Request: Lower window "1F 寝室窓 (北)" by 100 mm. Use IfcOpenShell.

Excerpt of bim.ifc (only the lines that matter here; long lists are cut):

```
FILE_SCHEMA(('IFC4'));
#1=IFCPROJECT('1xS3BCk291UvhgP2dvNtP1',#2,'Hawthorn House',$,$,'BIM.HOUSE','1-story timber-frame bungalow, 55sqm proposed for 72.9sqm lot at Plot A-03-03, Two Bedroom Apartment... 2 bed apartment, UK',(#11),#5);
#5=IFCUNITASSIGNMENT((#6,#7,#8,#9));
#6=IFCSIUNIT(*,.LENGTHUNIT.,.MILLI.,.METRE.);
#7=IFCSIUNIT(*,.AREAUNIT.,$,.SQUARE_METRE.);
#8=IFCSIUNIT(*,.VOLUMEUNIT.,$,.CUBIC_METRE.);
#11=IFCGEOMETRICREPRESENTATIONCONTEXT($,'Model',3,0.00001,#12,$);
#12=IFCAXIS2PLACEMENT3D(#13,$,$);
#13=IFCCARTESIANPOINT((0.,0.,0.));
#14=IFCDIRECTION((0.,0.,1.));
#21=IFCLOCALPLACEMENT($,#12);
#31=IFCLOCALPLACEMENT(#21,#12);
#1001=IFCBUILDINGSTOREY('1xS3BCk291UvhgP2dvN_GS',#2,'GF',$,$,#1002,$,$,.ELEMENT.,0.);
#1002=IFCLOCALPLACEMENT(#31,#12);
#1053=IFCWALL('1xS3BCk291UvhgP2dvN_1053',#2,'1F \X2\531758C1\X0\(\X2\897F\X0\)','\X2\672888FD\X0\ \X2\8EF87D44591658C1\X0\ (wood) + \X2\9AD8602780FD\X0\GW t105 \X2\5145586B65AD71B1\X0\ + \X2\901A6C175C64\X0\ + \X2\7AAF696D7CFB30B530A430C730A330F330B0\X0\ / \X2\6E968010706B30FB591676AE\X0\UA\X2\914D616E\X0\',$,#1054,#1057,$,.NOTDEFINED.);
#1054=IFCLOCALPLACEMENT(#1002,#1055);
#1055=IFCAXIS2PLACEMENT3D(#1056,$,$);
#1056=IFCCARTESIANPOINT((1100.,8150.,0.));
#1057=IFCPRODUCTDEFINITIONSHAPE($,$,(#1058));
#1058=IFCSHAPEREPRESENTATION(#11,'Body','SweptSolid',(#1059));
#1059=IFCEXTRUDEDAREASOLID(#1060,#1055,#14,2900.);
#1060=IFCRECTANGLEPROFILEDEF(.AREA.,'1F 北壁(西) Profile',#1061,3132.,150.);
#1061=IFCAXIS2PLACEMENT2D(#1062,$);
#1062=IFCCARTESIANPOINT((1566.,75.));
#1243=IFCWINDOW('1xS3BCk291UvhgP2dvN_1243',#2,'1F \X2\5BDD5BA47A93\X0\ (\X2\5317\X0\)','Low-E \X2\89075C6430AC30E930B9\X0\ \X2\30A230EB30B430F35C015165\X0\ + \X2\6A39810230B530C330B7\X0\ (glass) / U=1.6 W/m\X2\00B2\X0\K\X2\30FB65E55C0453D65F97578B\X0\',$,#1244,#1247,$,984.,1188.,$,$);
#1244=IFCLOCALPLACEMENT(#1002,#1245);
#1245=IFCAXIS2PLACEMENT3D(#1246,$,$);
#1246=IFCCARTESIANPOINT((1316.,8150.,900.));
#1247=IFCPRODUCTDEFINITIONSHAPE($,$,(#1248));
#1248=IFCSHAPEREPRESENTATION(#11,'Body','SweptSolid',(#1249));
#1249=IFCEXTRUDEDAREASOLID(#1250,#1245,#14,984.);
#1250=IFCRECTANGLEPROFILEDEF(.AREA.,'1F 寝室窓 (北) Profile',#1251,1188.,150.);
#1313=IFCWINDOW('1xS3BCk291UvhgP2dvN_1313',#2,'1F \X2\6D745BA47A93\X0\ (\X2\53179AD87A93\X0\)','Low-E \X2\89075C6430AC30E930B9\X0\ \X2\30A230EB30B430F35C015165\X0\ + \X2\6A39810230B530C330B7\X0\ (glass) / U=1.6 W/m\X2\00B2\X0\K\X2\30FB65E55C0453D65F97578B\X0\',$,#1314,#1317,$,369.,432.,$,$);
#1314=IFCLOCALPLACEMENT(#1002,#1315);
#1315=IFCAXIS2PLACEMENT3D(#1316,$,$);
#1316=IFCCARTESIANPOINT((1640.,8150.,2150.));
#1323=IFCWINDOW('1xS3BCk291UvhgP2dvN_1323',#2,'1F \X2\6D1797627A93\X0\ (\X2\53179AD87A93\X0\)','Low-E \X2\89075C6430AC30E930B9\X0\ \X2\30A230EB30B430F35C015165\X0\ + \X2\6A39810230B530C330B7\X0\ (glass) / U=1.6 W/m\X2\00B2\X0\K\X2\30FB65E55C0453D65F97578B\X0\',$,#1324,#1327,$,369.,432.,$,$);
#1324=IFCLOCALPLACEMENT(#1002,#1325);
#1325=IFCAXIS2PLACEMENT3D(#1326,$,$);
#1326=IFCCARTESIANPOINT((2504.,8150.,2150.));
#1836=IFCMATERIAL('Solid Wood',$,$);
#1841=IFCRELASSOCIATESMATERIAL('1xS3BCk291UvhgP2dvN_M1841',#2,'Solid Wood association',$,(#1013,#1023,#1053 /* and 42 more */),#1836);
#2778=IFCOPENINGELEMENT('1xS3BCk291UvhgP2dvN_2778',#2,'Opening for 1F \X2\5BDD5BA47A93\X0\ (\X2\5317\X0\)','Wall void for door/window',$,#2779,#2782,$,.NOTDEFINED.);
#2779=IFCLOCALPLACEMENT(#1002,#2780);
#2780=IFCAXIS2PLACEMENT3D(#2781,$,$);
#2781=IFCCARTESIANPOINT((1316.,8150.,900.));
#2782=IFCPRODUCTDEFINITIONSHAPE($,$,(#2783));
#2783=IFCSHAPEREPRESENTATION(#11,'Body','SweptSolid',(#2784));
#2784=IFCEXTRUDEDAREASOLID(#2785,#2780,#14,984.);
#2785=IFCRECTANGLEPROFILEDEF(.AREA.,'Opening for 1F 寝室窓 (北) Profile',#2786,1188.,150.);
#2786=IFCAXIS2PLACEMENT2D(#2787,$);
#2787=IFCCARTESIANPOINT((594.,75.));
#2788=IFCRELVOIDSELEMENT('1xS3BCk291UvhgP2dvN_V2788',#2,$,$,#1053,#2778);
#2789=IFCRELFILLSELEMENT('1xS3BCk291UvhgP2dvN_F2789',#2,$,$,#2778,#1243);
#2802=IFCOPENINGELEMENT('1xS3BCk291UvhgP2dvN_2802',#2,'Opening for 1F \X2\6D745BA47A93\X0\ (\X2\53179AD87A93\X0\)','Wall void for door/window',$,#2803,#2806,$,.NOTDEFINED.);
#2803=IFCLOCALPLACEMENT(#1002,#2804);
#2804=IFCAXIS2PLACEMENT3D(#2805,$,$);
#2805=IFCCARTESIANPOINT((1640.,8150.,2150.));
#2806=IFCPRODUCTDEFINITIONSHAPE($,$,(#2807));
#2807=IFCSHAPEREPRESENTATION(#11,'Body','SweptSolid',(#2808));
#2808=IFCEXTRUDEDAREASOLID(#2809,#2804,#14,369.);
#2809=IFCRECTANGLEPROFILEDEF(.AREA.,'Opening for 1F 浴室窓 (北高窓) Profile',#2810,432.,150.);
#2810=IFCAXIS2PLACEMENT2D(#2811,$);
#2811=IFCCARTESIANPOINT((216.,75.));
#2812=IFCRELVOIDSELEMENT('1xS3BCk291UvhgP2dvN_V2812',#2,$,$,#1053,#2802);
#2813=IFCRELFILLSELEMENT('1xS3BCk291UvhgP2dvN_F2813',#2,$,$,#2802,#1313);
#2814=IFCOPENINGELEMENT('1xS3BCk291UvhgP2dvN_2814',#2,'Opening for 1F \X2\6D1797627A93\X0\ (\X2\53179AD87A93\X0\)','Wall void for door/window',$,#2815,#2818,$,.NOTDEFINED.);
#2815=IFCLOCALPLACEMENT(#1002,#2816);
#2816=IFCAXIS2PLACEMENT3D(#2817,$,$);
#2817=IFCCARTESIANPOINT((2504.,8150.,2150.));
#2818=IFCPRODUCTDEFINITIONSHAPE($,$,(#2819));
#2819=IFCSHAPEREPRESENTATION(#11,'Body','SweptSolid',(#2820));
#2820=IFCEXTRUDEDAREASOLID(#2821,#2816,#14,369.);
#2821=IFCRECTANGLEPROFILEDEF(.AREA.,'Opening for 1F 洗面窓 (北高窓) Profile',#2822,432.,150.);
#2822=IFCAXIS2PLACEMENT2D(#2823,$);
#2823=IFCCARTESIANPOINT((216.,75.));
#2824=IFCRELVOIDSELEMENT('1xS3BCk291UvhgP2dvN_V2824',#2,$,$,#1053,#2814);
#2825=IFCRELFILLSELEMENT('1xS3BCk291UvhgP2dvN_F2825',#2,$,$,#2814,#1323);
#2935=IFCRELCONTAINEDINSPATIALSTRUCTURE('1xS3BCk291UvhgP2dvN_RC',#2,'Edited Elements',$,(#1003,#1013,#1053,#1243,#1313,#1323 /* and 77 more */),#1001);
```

```python
import numpy as np
import ifcopenshell
import ifcopenshell.api.geometry
import ifcopenshell.util.placement
import ifcopenshell.util.unit

model = ifcopenshell.open("bim.ifc")
unit_scale = ifcopenshell.util.unit.calculate_unit_scale(model)

window = model.by_guid("1xS3BCk291UvhgP2dvN_1243")
opening = window.FillsVoids[0].RelatingOpeningElement
dz = -0.1 / unit_scale

shift = np.array([0.0, 0.0, dz])
# The window is not placed relative to its opening, so move both.
for product in (opening, window):
    matrix = ifcopenshell.util.placement.get_local_placement(product.ObjectPlacement)
    matrix[:3, 3] += shift
    ifcopenshell.api.geometry.edit_object_placement(model, product=product, matrix=matrix, is_si=False)

print(f"moved by {dz * unit_scale:+.3f} m")

model.write("bim_rev.ifc")
```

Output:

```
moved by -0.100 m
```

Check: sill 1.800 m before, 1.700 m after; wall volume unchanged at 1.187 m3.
